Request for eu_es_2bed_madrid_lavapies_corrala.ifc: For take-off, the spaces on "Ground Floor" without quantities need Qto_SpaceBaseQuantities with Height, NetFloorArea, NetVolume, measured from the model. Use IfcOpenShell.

First a look at what the model holds.

```python
import ifcopenshell
import ifcopenshell.util.element
import ifcopenshell.util.unit

model = ifcopenshell.open("eu_es_2bed_madrid_lavapies_corrala.ifc")
print(model.schema)
for unit_type in ("LENGTHUNIT", "AREAUNIT", "VOLUMEUNIT"):
    print(unit_type, ifcopenshell.util.unit.calculate_unit_scale(model, unit_type))
storey = next(s for s in model.by_type("IfcBuildingStorey") if s.Name == "Ground Floor")
spaces = [e for e in ifcopenshell.util.element.get_decomposition(storey) if e.is_a("IfcSpace")]
for e in sorted(spaces, key=lambda e: e.id()):
    print(e.id(), e.is_a(), e.Name, list(ifcopenshell.util.element.get_psets(e, qtos_only=True)), sep=" | ")
```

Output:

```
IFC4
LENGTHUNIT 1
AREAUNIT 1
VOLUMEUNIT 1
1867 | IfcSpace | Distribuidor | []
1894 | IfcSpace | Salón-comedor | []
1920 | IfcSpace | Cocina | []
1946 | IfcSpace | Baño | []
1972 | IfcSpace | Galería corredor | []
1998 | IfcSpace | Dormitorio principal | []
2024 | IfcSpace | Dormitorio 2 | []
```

```python
import ifcopenshell
import ifcopenshell.api.pset
import ifcopenshell.geom
import ifcopenshell.util.element
import ifcopenshell.util.shape
import ifcopenshell.util.unit

model = ifcopenshell.open("eu_es_2bed_madrid_lavapies_corrala.ifc")
unit_scale = ifcopenshell.util.unit.calculate_unit_scale(model)
area_scale = ifcopenshell.util.unit.calculate_unit_scale(model, "AREAUNIT")
volume_scale = ifcopenshell.util.unit.calculate_unit_scale(model, "VOLUMEUNIT")
settings = ifcopenshell.geom.settings()

storey = next(s for s in model.by_type("IfcBuildingStorey") if s.Name == "Ground Floor")
spaces = [e for e in ifcopenshell.util.element.get_decomposition(storey) if e.is_a("IfcSpace")]

for e in sorted(spaces, key=lambda e: e.id()):
    if ifcopenshell.util.element.get_psets(e, qtos_only=True, should_inherit=False):
        continue
    # Geometry comes back in metres, in the element's own axes.
    shape = ifcopenshell.geom.create_shape(settings, e)
    values = {
        "Height": ifcopenshell.util.shape.get_z(shape.geometry) / unit_scale,
        "NetFloorArea": ifcopenshell.util.shape.get_footprint_area(shape.geometry) / area_scale,
        "NetVolume": ifcopenshell.util.shape.get_volume(shape.geometry) / volume_scale,
    }
    qto = ifcopenshell.api.pset.add_qto(model, product=e, name="Qto_SpaceBaseQuantities")
    ifcopenshell.api.pset.edit_qto(model, qto=qto, properties=values)
    print(e.id(), {k: round(v, 3) for k, v in values.items()})

model.write("eu_es_2bed_madrid_lavapies_corrala-out.ifc")
```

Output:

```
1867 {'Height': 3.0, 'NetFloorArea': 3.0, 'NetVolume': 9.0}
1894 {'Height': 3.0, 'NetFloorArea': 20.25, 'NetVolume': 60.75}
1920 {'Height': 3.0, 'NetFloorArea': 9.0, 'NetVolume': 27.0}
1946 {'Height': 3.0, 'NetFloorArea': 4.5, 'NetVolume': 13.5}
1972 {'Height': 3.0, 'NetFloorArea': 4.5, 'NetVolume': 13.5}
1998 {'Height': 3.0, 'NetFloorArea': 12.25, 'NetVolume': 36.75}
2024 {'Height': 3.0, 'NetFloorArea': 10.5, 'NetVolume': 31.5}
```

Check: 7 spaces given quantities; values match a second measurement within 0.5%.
